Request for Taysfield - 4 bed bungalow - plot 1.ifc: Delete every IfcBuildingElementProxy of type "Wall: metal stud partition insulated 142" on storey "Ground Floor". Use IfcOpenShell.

First a look at what the model holds.

```python
import ifcopenshell
import ifcopenshell.util.element

model = ifcopenshell.open("Taysfield - 4 bed bungalow - plot 1.ifc")
print(model.schema)
storey = next(s for s in model.by_type("IfcBuildingStorey") if s.Name == "Ground Floor")
proxies = [e for e in ifcopenshell.util.element.get_decomposition(storey) if e.is_a("IfcBuildingElementProxy")]
seen = {}
for e in proxies:
    element_type = ifcopenshell.util.element.get_type(e)
    name = element_type.Name if element_type not in (None, e) else None
    seen[name] = seen.get(name, 0) + 1
for name, count in sorted(seen.items(), key=str):
    print(count, "x", name)
```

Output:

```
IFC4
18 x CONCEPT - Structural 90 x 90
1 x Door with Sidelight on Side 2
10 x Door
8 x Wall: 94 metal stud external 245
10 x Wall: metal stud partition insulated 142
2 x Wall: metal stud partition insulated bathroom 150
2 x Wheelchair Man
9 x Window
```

```python
import ifcopenshell
import ifcopenshell.api.root
import ifcopenshell.util.element

model = ifcopenshell.open("Taysfield - 4 bed bungalow - plot 1.ifc")

storey = next(s for s in model.by_type("IfcBuildingStorey") if s.Name == "Ground Floor")
proxies = [e for e in ifcopenshell.util.element.get_decomposition(storey) if e.is_a("IfcBuildingElementProxy")]
targets = [e for e in proxies if (t := ifcopenshell.util.element.get_type(e)) not in (None, e) and t.Name == "Wall: metal stud partition insulated 142"]

for e in targets:
    ifcopenshell.api.root.remove_product(model, product=e)
print(len(targets), "removed")

model.write("Taysfield - 4 bed bungalow - plot 1_updated.ifc")
```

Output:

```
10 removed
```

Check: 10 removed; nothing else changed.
